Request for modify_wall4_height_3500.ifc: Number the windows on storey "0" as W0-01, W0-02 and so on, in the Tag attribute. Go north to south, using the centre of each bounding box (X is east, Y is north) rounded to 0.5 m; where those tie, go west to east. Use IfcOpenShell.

First a look at what the model holds.

```python
import ifcopenshell
import ifcopenshell.util.element
import ifcopenshell.util.placement

model = ifcopenshell.open("modify_wall4_height_3500.ifc")
print(model.schema)
storey = next(s for s in model.by_type("IfcBuildingStorey") if s.Name == "0")
windows = [e for e in ifcopenshell.util.element.get_decomposition(storey) if e.is_a("IfcWindow")]
for e in sorted(windows, key=lambda e: e.id()):
    origin = ifcopenshell.util.placement.get_local_placement(e.ObjectPlacement)[:3, 3]
    print(e.id(), e.Tag, e.Name, origin.round(2) + 0.0, sep=" | ")
```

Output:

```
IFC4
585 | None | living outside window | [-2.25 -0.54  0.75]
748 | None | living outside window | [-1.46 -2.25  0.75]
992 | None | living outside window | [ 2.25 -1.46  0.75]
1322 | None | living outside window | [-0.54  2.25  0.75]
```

```python
import ifcopenshell
import ifcopenshell.geom
import ifcopenshell.util.element
import ifcopenshell.util.shape

model = ifcopenshell.open("modify_wall4_height_3500.ifc")
settings = ifcopenshell.geom.settings()
settings.set("use-world-coords", True)


def centre(element):
    shape = ifcopenshell.geom.create_shape(settings, element)
    return ifcopenshell.util.shape.get_bbox_centroid(shape.geometry)


storey = next(s for s in model.by_type("IfcBuildingStorey") if s.Name == "0")
windows = [e for e in ifcopenshell.util.element.get_decomposition(storey) if e.is_a("IfcWindow")]

# Insertion points can sit at a corner or the storey origin, so sort by the geometry (in metres).
centres = {e: centre(e) for e in windows}
windows.sort(key=lambda e: (-round(centres[e][1] / 0.5), centres[e][0]))

for i, e in enumerate(windows, start=1):
    number = f"W0-{i:02d}"
    e.Tag = number
    print(e.id(), number)

model.write("modify_wall4_height_3500_edited.ifc")
```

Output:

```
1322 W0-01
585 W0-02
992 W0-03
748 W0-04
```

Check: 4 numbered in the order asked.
